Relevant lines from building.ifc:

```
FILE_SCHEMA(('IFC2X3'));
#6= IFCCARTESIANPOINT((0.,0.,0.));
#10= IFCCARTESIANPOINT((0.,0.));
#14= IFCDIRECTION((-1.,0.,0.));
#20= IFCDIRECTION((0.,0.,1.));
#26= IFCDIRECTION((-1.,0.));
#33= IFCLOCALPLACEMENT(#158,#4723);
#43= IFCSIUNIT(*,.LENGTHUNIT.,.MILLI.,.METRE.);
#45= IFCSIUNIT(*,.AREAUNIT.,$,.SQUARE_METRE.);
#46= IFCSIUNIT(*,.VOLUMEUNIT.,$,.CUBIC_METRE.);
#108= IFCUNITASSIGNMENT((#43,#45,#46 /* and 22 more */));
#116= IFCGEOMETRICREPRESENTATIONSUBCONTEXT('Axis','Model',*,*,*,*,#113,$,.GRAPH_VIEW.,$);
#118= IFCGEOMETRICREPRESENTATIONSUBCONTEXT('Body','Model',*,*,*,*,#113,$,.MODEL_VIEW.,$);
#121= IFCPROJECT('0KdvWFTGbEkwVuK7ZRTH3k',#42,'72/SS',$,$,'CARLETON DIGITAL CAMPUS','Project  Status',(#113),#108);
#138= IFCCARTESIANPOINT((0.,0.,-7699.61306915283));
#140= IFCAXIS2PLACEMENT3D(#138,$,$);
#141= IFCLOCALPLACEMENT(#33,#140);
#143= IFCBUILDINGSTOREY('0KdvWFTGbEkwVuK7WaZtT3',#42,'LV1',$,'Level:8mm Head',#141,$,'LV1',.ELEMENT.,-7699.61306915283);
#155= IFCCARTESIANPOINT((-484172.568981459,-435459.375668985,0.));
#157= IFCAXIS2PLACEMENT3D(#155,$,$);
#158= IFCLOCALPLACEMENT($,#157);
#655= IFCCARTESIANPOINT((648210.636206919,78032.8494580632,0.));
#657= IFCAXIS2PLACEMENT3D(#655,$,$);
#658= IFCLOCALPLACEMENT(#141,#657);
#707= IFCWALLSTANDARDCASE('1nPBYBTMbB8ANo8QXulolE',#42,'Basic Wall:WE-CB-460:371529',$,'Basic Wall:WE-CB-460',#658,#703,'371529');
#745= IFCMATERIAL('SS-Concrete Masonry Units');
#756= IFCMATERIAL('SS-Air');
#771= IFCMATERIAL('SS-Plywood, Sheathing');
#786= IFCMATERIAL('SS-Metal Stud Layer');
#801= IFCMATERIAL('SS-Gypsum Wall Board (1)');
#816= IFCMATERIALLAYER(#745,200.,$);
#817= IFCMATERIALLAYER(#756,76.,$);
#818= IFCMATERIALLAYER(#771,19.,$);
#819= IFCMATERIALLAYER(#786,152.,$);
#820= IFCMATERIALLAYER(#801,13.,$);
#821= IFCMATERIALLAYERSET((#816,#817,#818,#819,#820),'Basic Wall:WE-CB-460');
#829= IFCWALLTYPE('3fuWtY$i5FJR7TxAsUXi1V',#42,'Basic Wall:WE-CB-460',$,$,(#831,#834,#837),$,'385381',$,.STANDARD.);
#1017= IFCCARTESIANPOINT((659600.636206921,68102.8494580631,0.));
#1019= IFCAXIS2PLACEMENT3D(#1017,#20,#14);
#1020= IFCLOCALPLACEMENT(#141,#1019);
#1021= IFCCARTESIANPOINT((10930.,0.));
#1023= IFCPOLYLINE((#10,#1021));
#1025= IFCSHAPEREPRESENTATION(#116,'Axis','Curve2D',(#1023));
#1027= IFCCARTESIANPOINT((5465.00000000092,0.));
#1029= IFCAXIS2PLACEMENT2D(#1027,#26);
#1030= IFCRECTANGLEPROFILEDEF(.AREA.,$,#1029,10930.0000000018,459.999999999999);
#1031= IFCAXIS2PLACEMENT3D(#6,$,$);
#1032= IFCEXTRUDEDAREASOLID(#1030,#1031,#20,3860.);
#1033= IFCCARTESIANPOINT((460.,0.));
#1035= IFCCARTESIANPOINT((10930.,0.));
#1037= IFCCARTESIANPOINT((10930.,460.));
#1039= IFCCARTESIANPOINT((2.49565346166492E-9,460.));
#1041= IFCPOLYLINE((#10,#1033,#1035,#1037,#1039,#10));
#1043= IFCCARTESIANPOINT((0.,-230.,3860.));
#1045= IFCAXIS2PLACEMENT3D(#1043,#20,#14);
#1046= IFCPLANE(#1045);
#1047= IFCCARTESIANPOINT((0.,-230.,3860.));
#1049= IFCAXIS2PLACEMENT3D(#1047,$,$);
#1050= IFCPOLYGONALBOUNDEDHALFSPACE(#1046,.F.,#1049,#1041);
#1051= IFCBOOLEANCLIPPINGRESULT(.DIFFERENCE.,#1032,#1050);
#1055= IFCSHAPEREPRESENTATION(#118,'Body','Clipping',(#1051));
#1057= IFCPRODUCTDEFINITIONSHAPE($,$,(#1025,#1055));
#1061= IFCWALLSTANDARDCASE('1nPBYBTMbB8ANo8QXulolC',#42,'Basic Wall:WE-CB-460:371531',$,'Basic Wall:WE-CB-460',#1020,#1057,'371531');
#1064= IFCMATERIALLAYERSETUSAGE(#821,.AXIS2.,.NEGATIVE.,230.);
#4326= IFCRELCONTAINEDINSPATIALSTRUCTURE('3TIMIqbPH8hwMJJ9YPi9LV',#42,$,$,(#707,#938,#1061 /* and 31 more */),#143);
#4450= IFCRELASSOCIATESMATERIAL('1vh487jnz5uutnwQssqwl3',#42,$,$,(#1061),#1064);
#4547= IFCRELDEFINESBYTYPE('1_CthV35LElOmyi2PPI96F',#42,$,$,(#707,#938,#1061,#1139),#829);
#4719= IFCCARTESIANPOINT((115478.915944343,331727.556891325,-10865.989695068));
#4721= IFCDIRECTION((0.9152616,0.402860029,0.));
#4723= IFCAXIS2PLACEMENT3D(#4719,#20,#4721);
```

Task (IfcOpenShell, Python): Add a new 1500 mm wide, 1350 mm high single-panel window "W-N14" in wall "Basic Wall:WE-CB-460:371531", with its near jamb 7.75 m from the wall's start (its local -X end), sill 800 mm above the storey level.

```python
import numpy as np
import ifcopenshell
import ifcopenshell.api.feature
import ifcopenshell.api.geometry
import ifcopenshell.api.root
import ifcopenshell.api.spatial
import ifcopenshell.api.type
import ifcopenshell.geom
import ifcopenshell.util.element
import ifcopenshell.util.placement
import ifcopenshell.util.representation
import ifcopenshell.util.shape
import ifcopenshell.util.unit

model = ifcopenshell.open("building.ifc")
unit_scale = ifcopenshell.util.unit.calculate_unit_scale(model)
settings = ifcopenshell.geom.settings()


def volume(element):
    """Net volume in cubic metres, openings subtracted."""
    shape = ifcopenshell.geom.create_shape(settings, element)
    return ifcopenshell.util.shape.get_volume(shape.geometry)


wall = model.by_guid("1nPBYBTMbB8ANo8QXulolC")
storey = ifcopenshell.util.element.get_container(wall, ifc_class="IfcBuildingStorey")
context = ifcopenshell.util.representation.get_context(model, "Model", "Body", "MODEL_VIEW")
before = volume(wall)

width, height, from_end, sill = 1.5, 1.35, 7.75, 0.8  # metres

# The wall runs along its own X axis, and the end named is its -X end.
wall_shape = ifcopenshell.geom.create_shape(settings, wall)
x, y, z = ifcopenshell.util.shape.get_vertices(wall_shape.geometry).T
start = x.min() + from_end
face, thickness = float(y.min()), float(y.max() - y.min())
wall_matrix = ifcopenshell.util.placement.get_local_placement(wall.ObjectPlacement)
level = ifcopenshell.util.placement.get_local_placement(storey.ObjectPlacement)[2, 3]


def in_wall(x, y):
    """Placement at x, y metres in the wall's axes, at sill height."""
    matrix = wall_matrix.copy()
    matrix[:, 3] = wall_matrix @ np.array([x / unit_scale, y / unit_scale, 0.0, 1.0])
    matrix[2, 3] = level + sill / unit_scale
    return matrix


# Opening: a box that overshoots both wall faces by 50 mm.
opening = ifcopenshell.api.root.create_entity(model, ifc_class="IfcOpeningElement")
box = ifcopenshell.api.geometry.add_wall_representation(
    model, context=context, length=width, height=height, thickness=thickness + 0.1
)
ifcopenshell.api.geometry.assign_representation(model, product=opening, representation=box)
ifcopenshell.api.geometry.edit_object_placement(model, product=opening, matrix=in_wall(start, face - 0.05), is_si=False)
ifcopenshell.api.feature.add_feature(model, feature=opening, element=wall)

window = ifcopenshell.api.root.create_entity(model, ifc_class="IfcWindow", name="W-N14")
window.OverallWidth, window.OverallHeight = width / unit_scale, height / unit_scale
body = ifcopenshell.api.geometry.add_window_representation(
    model,
    context=context,
    overall_width=window.OverallWidth,
    overall_height=window.OverallHeight,
    partition_type="SINGLE_PANEL",
)
ifcopenshell.api.geometry.assign_representation(model, product=window, representation=body)
ifcopenshell.api.spatial.assign_container(model, products=[window], relating_structure=storey)
fills = ifcopenshell.api.feature.add_filling(model, opening=opening, element=window)
fills.OwnerHistory = window.OwnerHistory  # required in IFC2X3

# IFC2X3 keeps the operation on the window style.
style = ifcopenshell.api.root.create_entity(model, ifc_class="IfcWindowStyle", name="W-N14")
style.OperationType, style.ConstructionType = "SINGLE_PANEL", "NOTDEFINED"
style.ParameterTakesPrecedence = style.Sizeable = False
ifcopenshell.api.type.assign_type(model, related_objects=[window], relating_type=style)

# Centre the window in the wall's thickness.
ifcopenshell.api.geometry.edit_object_placement(model, product=window, matrix=in_wall(start, face), is_si=False)
window_shape = ifcopenshell.geom.create_shape(settings, window)
depth = ifcopenshell.util.shape.get_vertices(window_shape.geometry)[:, 1]
offset = face + thickness / 2 - (depth.min() + depth.max()) / 2
ifcopenshell.api.geometry.edit_object_placement(model, product=window, matrix=in_wall(start, offset), is_si=False)

after = volume(wall)

print(f"wall volume {before:.3f} -> {after:.3f} m3")

model.write("building_updated.ifc")
```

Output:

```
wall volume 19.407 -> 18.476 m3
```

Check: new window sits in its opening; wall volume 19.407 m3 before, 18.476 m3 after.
